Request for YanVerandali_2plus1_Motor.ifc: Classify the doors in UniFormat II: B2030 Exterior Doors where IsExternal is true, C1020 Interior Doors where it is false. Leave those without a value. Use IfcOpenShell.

First a look at what the model holds.

```python
import ifcopenshell
import ifcopenshell.util.element

model = ifcopenshell.open("YanVerandali_2plus1_Motor.ifc")
print(model.schema)
print("classifications:", [c.Name for c in model.by_type("IfcClassification")])
values = [ifcopenshell.util.element.get_pset(e, "Pset_DoorCommon", "IsExternal") for e in model.by_type("IfcDoor")]
for value in (True, False, None):
    print("IsExternal", value, values.count(value))
```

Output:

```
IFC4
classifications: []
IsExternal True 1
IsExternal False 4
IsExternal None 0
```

```python
import ifcopenshell
import ifcopenshell.api.classification
import ifcopenshell.util.element

model = ifcopenshell.open("YanVerandali_2plus1_Motor.ifc")

system = ifcopenshell.api.classification.add_classification(model, classification="UniFormat II")

doors = model.by_type("IfcDoor")
external = {e: ifcopenshell.util.element.get_pset(e, "Pset_DoorCommon", "IsExternal") for e in doors}
for flag, code, name in ((True, "B2030", "Exterior Doors"), (False, "C1020", "Interior Doors")):
    products = [e for e in doors if external[e] is flag]
    ifcopenshell.api.classification.add_reference(
        model, products=products, classification=system, identification=code, name=name
    )
    print(code, len(products))

model.write("YanVerandali_2plus1_Motor_v2.ifc")
```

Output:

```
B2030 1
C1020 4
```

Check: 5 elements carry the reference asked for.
